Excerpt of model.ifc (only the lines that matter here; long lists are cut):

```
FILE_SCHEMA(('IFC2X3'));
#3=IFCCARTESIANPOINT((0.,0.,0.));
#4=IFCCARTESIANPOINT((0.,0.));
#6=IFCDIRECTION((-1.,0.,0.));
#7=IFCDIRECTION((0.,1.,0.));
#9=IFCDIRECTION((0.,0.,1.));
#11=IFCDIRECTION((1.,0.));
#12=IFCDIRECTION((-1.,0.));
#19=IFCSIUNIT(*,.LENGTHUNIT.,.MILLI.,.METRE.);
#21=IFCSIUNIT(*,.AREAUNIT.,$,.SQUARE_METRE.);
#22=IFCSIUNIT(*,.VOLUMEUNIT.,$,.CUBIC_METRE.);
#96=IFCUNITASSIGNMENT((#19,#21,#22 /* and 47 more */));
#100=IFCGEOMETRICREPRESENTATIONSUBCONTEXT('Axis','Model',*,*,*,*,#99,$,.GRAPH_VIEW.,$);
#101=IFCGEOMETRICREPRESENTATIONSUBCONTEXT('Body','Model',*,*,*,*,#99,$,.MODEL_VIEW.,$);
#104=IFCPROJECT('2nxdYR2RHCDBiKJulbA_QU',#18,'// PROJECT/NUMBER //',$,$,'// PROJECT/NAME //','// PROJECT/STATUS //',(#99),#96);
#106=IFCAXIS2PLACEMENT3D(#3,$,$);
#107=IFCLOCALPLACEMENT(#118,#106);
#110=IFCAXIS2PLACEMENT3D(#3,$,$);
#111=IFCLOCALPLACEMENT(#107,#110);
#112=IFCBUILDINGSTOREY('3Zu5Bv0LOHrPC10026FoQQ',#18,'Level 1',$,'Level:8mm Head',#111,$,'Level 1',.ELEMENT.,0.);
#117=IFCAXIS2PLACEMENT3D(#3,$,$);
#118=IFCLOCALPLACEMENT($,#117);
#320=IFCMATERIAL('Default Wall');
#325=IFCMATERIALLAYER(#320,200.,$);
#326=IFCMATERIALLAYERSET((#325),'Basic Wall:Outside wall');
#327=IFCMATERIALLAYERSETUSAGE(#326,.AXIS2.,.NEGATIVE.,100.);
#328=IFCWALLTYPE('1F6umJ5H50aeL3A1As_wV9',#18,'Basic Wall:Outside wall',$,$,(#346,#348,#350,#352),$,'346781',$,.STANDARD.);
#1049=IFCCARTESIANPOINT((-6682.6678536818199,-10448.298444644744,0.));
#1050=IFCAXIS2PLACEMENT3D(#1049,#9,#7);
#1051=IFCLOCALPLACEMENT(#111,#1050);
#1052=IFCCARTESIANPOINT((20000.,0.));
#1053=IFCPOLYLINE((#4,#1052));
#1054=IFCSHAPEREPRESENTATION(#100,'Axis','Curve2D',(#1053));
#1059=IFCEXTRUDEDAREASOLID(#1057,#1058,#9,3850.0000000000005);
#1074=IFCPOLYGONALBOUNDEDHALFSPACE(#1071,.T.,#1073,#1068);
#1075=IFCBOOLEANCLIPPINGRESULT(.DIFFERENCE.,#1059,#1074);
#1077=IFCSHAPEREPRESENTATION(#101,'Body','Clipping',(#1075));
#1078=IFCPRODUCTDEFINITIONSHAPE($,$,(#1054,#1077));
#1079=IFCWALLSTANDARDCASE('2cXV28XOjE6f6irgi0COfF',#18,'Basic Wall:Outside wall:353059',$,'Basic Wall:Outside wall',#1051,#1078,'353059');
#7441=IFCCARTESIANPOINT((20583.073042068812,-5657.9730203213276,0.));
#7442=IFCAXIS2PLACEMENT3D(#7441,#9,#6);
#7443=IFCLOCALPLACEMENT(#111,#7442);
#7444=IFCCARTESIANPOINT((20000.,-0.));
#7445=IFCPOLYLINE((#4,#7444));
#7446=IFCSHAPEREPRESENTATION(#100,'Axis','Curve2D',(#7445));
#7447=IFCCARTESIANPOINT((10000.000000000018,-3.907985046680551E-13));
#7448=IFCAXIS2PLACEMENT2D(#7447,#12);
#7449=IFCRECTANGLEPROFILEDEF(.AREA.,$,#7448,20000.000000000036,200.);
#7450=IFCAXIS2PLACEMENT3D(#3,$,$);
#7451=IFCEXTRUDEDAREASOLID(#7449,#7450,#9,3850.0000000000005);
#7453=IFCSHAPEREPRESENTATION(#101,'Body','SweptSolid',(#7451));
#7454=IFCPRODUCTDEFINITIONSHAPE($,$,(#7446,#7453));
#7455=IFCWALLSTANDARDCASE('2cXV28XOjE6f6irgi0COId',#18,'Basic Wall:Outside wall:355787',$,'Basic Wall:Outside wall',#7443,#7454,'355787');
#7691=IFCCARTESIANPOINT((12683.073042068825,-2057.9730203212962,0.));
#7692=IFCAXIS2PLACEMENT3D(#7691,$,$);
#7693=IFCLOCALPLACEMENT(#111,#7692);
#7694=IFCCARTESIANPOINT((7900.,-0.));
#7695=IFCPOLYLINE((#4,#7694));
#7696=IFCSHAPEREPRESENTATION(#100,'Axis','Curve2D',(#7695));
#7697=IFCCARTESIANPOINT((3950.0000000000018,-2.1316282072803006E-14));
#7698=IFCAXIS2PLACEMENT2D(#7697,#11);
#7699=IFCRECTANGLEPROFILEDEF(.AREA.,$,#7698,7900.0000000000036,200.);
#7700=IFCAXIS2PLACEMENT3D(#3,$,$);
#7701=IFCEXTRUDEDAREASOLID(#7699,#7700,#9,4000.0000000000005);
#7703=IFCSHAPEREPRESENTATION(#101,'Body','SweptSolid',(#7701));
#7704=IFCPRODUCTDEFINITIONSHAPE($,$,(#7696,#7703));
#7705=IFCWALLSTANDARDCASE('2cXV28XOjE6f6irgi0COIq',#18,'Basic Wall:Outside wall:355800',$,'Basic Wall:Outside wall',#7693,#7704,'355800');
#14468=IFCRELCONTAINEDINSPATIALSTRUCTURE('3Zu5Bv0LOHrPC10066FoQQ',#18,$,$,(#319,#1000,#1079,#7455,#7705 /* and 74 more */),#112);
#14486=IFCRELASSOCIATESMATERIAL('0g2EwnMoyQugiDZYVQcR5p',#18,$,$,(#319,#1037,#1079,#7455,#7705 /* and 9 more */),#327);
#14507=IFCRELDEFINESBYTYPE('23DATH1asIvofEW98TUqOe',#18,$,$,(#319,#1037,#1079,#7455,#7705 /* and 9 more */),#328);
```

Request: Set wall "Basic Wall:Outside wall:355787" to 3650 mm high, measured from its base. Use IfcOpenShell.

```python
import ifcopenshell
import ifcopenshell.geom
import ifcopenshell.util.representation
import ifcopenshell.util.shape
import ifcopenshell.util.unit

model = ifcopenshell.open("model.ifc")
unit_scale = ifcopenshell.util.unit.calculate_unit_scale(model)
settings = ifcopenshell.geom.settings()


def volume(element):
    """Net volume in cubic metres, openings subtracted."""
    shape = ifcopenshell.geom.create_shape(settings, element)
    return ifcopenshell.util.shape.get_volume(shape.geometry)


wall = model.by_guid("2cXV28XOjE6f6irgi0COId")
before = volume(wall)

body = ifcopenshell.util.representation.get_representation(wall, "Model", "Body")
solid = body.Items[0]
old_height = solid.Depth
solid.Depth = 3.65 / unit_scale
after = volume(wall)

print(f"height {old_height:g} -> {solid.Depth:g}, volume {before:.3f} -> {after:.3f} m3")

model.write("model-out.ifc")
```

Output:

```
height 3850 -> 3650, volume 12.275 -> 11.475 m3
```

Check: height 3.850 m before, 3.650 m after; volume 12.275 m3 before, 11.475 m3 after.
